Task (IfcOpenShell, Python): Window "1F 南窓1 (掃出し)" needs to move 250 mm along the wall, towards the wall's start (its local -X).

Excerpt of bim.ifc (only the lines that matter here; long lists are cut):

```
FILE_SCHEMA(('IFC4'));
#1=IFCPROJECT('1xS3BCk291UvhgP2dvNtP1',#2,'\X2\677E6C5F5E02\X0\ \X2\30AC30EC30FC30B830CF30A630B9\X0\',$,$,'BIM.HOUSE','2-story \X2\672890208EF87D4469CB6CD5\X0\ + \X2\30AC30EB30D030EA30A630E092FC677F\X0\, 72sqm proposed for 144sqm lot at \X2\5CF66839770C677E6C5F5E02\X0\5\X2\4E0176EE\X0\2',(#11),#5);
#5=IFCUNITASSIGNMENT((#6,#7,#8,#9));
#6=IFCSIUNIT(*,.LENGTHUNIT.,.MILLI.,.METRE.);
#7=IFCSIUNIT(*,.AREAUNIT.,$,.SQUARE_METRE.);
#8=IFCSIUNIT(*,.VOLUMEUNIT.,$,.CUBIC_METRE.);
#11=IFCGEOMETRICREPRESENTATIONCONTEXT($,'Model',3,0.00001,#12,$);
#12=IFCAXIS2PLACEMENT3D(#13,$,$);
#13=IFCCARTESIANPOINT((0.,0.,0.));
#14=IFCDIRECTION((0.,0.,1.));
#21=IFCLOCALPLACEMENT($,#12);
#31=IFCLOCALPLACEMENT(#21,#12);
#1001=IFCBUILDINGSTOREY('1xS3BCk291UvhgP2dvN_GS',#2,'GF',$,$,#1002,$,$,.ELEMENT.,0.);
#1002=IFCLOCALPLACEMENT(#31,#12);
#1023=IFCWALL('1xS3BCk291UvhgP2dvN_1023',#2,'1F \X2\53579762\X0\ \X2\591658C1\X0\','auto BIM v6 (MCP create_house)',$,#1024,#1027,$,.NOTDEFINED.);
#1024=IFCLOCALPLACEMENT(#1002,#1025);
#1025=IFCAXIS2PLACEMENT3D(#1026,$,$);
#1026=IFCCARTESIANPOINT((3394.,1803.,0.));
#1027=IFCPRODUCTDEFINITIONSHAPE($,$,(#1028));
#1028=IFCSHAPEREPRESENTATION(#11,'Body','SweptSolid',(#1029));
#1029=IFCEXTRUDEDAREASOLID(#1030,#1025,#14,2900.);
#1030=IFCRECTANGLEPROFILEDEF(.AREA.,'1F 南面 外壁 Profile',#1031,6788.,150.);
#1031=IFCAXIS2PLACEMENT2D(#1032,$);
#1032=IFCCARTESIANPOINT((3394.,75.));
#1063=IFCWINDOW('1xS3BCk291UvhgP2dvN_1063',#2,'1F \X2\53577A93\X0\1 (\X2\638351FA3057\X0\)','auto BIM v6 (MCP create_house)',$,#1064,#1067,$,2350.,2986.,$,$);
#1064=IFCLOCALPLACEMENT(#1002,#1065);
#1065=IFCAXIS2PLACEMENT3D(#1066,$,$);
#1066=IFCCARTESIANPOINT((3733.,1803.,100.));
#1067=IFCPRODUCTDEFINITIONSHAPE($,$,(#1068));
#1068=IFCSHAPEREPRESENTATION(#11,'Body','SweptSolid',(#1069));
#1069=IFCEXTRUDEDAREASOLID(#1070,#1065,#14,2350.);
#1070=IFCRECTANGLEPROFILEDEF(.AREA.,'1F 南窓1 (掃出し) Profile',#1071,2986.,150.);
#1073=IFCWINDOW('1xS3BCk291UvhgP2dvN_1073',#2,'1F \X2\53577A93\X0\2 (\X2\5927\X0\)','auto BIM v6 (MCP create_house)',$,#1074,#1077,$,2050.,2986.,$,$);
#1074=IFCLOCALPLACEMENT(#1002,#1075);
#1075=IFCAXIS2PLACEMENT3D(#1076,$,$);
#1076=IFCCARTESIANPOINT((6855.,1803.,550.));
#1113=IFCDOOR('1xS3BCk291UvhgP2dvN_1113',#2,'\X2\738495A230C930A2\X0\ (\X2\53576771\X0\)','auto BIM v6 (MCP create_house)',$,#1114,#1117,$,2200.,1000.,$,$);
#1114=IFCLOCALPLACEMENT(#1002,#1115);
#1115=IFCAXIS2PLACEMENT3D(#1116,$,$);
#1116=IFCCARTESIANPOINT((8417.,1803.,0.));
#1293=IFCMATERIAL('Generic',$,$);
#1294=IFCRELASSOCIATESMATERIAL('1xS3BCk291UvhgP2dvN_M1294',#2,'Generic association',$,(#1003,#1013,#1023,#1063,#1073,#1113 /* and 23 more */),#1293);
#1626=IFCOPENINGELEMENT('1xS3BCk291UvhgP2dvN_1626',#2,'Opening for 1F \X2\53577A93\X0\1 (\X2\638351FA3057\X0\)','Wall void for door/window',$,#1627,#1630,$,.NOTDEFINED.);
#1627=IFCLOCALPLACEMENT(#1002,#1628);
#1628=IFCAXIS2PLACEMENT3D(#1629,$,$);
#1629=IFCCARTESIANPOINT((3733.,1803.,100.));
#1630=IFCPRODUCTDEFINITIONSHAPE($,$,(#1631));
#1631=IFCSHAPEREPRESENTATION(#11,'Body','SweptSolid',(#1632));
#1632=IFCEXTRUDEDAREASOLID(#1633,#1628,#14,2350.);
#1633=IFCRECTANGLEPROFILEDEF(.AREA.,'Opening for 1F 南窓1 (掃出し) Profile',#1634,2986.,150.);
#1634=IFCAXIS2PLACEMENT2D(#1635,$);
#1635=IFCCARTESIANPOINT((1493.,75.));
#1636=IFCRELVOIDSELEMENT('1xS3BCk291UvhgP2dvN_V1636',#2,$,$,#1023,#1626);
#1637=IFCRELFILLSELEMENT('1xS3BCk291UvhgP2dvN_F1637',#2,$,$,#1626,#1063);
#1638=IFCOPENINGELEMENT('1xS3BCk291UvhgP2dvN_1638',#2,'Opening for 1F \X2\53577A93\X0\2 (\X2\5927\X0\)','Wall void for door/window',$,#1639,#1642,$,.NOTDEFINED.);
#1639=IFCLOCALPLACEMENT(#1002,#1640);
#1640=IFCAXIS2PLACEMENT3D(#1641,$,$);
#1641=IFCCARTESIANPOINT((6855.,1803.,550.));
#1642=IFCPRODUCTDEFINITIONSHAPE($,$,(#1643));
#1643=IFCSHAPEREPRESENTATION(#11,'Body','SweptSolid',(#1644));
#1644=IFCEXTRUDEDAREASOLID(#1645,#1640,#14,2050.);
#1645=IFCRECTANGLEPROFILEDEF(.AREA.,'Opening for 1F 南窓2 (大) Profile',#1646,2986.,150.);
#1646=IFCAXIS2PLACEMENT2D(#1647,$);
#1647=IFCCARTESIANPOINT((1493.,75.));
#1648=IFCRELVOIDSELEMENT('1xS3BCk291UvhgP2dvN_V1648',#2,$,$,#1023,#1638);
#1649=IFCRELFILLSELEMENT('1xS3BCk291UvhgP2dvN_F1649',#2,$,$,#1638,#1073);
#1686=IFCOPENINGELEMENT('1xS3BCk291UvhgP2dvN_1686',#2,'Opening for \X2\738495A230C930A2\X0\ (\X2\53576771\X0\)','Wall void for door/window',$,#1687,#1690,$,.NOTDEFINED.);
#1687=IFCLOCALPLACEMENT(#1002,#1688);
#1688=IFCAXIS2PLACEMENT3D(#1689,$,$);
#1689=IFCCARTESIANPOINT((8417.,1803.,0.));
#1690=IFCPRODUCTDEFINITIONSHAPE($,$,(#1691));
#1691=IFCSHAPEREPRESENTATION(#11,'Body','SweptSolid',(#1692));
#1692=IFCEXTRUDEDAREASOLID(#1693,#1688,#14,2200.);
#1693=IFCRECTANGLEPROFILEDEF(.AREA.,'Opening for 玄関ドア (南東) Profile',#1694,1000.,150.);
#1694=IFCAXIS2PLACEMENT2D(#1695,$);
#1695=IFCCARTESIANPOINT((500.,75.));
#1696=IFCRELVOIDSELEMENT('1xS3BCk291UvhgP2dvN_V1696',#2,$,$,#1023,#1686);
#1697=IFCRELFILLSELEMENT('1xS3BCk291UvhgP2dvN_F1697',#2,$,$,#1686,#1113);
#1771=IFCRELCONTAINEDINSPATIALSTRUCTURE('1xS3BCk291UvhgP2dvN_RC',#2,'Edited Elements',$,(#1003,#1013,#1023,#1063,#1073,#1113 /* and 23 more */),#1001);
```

```python
import ifcopenshell
import ifcopenshell.api.geometry
import ifcopenshell.util.placement

model = ifcopenshell.open("bim.ifc")

window = model.by_guid("1xS3BCk291UvhgP2dvN_1063")
opening = window.FillsVoids[0].RelatingOpeningElement
wall = opening.VoidsElements[0].RelatingBuildingElement

wall_matrix = ifcopenshell.util.placement.get_local_placement(wall.ObjectPlacement)
shift = wall_matrix[:3, 0] * -250.0
before = ifcopenshell.util.placement.get_local_placement(window.ObjectPlacement)[:3, 3].copy()

# The window is not placed relative to its opening, so move both.
for product in (opening, window):
    matrix = ifcopenshell.util.placement.get_local_placement(product.ObjectPlacement)
    matrix[:3, 3] += shift
    ifcopenshell.api.geometry.edit_object_placement(model, product=product, matrix=matrix, is_si=False)

after = ifcopenshell.util.placement.get_local_placement(window.ObjectPlacement)[:3, 3]
print("window moved by", (after - before).round(3) + 0.0)

model.write("bim_edited.ifc")
```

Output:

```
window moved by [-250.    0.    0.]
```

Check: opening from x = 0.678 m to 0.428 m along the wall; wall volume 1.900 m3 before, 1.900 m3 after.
